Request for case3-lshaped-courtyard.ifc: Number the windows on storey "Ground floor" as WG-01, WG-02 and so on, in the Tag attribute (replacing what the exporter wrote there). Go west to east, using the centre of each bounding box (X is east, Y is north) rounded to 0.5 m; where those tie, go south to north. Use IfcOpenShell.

First a look at what the model holds.

```python
import ifcopenshell
import ifcopenshell.util.element
import ifcopenshell.util.placement

model = ifcopenshell.open("case3-lshaped-courtyard.ifc")
print(model.schema)
storey = next(s for s in model.by_type("IfcBuildingStorey") if s.Name == "Ground floor")
windows = [e for e in ifcopenshell.util.element.get_decomposition(storey) if e.is_a("IfcWindow")]
for e in sorted(windows, key=lambda e: e.id()):
    origin = ifcopenshell.util.placement.get_local_placement(e.ObjectPlacement)[:3, 3]
    print(e.id(), e.Tag, e.Name, origin.round(2) + 0.0, sep=" | ")
```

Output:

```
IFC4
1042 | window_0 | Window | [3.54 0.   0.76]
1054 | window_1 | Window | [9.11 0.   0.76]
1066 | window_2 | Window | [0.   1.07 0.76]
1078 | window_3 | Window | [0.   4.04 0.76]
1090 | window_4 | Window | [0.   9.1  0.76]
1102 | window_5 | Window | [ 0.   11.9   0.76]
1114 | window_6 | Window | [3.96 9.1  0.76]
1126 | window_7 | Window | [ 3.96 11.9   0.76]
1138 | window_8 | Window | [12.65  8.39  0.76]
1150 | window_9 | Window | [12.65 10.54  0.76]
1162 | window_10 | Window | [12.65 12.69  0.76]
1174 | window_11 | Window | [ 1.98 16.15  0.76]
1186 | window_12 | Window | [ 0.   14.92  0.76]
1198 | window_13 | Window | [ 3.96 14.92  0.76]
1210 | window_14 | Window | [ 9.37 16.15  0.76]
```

```python
import ifcopenshell
import ifcopenshell.geom
import ifcopenshell.util.element
import ifcopenshell.util.shape

model = ifcopenshell.open("case3-lshaped-courtyard.ifc")
settings = ifcopenshell.geom.settings()
settings.set("use-world-coords", True)


def centre(element):
    shape = ifcopenshell.geom.create_shape(settings, element)
    return ifcopenshell.util.shape.get_bbox_centroid(shape.geometry)


storey = next(s for s in model.by_type("IfcBuildingStorey") if s.Name == "Ground floor")
windows = [e for e in ifcopenshell.util.element.get_decomposition(storey) if e.is_a("IfcWindow")]

# Insertion points can sit at a corner or the storey origin, so sort by the geometry (in metres).
centres = {e: centre(e) for e in windows}
windows.sort(key=lambda e: (round(centres[e][0] / 0.5), centres[e][1]))

for i, e in enumerate(windows, start=1):
    number = f"WG-{i:02d}"
    e.Tag = number
    print(e.id(), number)

model.write("case3-lshaped-courtyard-out.ifc")
```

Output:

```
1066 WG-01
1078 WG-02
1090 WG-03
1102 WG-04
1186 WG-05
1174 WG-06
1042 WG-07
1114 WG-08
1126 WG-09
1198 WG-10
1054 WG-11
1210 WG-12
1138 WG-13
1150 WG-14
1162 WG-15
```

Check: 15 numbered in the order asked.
